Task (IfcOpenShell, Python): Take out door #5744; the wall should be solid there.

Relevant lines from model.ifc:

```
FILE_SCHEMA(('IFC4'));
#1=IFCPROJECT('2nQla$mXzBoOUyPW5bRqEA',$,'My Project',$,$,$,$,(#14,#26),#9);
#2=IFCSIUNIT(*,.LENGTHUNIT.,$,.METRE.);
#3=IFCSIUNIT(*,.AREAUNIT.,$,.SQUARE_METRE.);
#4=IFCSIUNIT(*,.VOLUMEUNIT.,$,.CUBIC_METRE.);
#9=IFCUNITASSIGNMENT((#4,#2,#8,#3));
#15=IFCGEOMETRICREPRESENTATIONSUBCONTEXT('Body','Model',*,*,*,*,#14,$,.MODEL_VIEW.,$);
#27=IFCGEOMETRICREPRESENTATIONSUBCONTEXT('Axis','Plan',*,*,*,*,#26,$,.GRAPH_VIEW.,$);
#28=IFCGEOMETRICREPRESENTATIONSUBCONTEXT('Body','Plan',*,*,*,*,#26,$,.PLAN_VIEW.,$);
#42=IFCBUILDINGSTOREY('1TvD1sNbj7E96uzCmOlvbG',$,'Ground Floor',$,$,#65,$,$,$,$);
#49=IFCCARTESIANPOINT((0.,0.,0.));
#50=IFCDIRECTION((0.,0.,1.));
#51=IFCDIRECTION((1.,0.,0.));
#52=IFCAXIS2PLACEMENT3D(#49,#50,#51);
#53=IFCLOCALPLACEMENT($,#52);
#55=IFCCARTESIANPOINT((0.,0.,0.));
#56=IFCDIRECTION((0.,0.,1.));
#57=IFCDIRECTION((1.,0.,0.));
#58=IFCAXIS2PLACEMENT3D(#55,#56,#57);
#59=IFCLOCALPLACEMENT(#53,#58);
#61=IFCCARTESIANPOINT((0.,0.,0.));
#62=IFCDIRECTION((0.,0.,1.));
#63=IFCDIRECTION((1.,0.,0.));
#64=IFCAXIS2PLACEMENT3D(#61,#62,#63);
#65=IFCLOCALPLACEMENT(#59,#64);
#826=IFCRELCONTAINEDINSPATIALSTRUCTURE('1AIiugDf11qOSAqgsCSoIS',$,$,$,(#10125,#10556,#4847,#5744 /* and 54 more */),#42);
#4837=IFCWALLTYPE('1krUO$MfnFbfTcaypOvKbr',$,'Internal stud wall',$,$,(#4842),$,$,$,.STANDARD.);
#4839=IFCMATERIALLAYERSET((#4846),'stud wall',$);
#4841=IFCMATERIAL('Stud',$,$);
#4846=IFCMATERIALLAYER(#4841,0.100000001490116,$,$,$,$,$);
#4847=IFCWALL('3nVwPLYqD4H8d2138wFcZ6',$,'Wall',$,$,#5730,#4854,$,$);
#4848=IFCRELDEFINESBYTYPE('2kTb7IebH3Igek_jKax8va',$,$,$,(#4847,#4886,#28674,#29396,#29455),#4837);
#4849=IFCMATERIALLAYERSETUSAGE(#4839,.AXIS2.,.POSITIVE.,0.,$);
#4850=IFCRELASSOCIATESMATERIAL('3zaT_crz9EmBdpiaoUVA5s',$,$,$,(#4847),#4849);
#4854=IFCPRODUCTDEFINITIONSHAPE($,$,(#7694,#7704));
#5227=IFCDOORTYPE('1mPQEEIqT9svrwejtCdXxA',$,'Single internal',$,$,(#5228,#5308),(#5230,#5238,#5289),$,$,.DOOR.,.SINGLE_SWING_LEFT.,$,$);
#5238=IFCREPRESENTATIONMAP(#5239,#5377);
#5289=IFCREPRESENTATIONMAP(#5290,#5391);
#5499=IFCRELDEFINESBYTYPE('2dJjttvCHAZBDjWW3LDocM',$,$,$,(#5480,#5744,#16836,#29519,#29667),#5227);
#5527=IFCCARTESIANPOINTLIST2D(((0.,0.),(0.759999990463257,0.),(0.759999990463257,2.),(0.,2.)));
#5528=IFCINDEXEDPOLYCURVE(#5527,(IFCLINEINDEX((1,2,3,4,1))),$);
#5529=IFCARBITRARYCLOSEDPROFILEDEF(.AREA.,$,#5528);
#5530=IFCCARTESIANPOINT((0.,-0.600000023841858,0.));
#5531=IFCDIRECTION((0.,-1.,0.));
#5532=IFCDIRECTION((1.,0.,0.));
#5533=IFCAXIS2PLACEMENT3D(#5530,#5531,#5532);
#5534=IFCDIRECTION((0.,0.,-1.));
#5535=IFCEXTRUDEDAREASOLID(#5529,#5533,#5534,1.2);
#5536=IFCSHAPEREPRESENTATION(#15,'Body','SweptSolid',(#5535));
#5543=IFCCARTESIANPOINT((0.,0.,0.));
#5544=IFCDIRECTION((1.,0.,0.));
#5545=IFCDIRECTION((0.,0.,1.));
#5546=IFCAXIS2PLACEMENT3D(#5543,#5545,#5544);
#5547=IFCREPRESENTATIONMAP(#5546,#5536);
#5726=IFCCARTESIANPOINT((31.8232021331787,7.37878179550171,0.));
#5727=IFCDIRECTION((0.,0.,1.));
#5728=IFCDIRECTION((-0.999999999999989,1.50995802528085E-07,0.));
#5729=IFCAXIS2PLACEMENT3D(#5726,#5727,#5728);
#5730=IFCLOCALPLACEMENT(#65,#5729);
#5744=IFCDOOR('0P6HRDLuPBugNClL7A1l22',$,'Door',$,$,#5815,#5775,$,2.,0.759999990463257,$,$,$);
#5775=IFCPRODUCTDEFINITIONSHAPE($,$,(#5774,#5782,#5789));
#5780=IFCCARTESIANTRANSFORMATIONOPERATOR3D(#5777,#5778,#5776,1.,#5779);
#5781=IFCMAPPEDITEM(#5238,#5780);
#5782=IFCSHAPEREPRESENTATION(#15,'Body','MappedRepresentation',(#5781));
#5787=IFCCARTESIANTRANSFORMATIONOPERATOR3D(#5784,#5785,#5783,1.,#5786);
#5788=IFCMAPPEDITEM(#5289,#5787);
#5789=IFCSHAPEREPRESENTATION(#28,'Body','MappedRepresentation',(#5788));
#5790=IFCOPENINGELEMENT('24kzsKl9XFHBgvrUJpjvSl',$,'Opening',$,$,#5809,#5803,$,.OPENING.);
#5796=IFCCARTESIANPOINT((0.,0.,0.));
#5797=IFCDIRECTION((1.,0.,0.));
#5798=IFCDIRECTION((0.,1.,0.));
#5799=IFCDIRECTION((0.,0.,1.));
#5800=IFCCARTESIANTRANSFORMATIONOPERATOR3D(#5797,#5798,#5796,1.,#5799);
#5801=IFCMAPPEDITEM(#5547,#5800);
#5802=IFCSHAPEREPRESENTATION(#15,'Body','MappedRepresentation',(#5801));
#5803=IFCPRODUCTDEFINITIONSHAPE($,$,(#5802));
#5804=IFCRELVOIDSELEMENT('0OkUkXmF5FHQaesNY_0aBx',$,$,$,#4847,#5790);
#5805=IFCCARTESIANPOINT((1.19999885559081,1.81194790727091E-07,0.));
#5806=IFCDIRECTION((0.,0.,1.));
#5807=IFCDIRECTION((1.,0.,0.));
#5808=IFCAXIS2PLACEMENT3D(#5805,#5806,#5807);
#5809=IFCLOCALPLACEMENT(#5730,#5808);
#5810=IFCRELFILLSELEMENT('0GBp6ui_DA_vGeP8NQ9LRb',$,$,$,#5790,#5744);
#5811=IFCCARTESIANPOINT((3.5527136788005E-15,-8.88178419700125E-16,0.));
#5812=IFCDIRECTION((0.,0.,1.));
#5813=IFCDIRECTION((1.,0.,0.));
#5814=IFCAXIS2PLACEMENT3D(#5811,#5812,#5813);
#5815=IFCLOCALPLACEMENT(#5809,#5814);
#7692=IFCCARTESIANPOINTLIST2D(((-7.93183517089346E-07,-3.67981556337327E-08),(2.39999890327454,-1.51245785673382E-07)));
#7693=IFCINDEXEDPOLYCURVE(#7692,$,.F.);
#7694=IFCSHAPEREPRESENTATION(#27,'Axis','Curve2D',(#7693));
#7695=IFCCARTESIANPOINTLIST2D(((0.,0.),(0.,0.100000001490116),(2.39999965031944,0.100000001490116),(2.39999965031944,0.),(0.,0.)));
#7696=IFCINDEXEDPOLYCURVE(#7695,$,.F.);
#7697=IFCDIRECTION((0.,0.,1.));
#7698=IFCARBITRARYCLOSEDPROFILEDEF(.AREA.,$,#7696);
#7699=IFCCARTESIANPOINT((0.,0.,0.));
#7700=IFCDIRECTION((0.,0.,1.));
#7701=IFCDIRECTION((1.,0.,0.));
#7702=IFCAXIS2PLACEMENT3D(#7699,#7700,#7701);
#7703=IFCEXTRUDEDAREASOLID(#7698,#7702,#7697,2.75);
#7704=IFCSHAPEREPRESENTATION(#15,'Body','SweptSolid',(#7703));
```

```python
import ifcopenshell
import ifcopenshell.api.feature
import ifcopenshell.api.root
import ifcopenshell.geom
import ifcopenshell.util.shape

model = ifcopenshell.open("model.ifc")
settings = ifcopenshell.geom.settings()


def volume(element):
    """Net volume in cubic metres, openings subtracted."""
    shape = ifcopenshell.geom.create_shape(settings, element)
    return ifcopenshell.util.shape.get_volume(shape.geometry)


door = model.by_id(5744)
opening = door.FillsVoids[0].RelatingOpeningElement
wall = opening.VoidsElements[0].RelatingBuildingElement
before = volume(wall)

ifcopenshell.api.root.remove_product(model, product=door)
ifcopenshell.api.feature.remove_feature(model, feature=opening)

after = volume(wall)

print(f"wall volume {before:.3f} -> {after:.3f} m3")

model.write("model_rev.ifc")
```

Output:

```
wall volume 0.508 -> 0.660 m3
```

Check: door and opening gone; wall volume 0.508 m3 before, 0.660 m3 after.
